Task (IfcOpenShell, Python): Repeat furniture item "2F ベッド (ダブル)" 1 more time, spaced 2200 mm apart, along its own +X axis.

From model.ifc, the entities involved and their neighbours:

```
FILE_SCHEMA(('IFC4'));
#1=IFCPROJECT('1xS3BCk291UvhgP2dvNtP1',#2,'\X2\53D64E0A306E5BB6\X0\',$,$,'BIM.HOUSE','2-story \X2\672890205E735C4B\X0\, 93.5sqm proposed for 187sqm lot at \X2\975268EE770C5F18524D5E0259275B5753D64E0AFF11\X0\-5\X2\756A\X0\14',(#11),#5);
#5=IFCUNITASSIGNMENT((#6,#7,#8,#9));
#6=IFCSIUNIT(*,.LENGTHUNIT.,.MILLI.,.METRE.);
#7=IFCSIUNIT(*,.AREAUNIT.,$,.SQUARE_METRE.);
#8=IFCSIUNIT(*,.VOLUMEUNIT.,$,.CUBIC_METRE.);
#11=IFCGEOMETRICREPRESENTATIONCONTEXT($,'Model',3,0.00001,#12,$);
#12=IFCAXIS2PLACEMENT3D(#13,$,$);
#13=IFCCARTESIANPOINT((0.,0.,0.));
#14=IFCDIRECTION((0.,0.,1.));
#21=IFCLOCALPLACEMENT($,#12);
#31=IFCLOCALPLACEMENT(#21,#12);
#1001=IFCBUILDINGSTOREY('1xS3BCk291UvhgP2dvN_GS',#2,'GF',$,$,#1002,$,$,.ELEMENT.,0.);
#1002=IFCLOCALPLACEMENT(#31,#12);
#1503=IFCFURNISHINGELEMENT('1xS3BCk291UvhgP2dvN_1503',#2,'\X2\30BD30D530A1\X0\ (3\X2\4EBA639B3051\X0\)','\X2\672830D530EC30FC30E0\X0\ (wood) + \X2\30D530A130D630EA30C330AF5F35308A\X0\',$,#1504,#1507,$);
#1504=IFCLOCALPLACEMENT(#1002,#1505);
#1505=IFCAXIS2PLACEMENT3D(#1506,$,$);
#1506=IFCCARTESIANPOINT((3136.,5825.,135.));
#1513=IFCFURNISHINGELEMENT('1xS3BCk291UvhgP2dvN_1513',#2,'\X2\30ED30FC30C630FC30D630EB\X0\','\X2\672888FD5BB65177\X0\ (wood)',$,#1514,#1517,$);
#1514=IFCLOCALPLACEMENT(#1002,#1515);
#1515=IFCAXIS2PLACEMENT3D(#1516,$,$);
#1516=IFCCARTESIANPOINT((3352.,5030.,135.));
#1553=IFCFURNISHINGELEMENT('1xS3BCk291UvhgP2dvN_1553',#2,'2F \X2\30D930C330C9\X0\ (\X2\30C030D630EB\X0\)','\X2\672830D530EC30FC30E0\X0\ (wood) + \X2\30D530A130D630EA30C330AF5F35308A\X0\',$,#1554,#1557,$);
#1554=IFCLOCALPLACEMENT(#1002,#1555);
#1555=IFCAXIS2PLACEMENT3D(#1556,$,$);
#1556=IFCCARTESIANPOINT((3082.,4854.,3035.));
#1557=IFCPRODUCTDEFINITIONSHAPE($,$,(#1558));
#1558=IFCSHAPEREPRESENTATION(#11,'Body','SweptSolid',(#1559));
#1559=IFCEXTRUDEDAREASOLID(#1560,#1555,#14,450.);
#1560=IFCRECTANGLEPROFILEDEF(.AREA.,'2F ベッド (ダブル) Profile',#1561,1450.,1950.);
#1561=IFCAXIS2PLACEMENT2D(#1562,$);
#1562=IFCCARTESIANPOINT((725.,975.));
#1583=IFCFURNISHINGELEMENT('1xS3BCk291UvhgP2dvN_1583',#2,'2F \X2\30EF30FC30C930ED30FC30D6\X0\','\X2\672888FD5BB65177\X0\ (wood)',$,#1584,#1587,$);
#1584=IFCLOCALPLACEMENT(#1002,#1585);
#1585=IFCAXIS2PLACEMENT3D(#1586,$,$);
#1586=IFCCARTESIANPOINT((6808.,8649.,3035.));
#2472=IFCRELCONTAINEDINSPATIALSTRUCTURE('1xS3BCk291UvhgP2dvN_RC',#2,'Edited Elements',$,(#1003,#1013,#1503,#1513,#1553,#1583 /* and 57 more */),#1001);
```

```python
import ifcopenshell
import ifcopenshell.api.geometry
import ifcopenshell.api.root
import ifcopenshell.util.element
import ifcopenshell.util.placement
import ifcopenshell.util.unit

model = ifcopenshell.open("model.ifc")
unit_scale = ifcopenshell.util.unit.calculate_unit_scale(model)


def reuse_history(source, copy):
    """copy_class also copies each property set's owner history, people and application; keep the originals."""
    for rel in copy.IsDefinedBy:
        if rel.is_a("IfcRelDefinesByProperties") and (history := rel.RelatingPropertyDefinition.OwnerHistory):
            rel.RelatingPropertyDefinition.OwnerHistory = source.OwnerHistory
            ifcopenshell.util.element.remove_deep2(model, history)


source = model.by_guid("1xS3BCk291UvhgP2dvN_1553")
base = ifcopenshell.util.placement.get_local_placement(source.ObjectPlacement)
step = base[:3, 0] * 2.2 / unit_scale

for i in range(1, 2):
    copy = ifcopenshell.api.root.copy_class(model, product=source)
    copy.Representation = ifcopenshell.util.element.copy_deep(
        model, source.Representation, exclude=["IfcGeometricRepresentationContext", "IfcRepresentationMap"]
    )
    reuse_history(source, copy)
    matrix = base.copy()
    matrix[:3, 3] += i * step
    print("added at", matrix[:3, 3].round(3) + 0.0)
    ifcopenshell.api.geometry.edit_object_placement(model, product=copy, matrix=matrix, is_si=False)

model.write("model-out.ifc")
```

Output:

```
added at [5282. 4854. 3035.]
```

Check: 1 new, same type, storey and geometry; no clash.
